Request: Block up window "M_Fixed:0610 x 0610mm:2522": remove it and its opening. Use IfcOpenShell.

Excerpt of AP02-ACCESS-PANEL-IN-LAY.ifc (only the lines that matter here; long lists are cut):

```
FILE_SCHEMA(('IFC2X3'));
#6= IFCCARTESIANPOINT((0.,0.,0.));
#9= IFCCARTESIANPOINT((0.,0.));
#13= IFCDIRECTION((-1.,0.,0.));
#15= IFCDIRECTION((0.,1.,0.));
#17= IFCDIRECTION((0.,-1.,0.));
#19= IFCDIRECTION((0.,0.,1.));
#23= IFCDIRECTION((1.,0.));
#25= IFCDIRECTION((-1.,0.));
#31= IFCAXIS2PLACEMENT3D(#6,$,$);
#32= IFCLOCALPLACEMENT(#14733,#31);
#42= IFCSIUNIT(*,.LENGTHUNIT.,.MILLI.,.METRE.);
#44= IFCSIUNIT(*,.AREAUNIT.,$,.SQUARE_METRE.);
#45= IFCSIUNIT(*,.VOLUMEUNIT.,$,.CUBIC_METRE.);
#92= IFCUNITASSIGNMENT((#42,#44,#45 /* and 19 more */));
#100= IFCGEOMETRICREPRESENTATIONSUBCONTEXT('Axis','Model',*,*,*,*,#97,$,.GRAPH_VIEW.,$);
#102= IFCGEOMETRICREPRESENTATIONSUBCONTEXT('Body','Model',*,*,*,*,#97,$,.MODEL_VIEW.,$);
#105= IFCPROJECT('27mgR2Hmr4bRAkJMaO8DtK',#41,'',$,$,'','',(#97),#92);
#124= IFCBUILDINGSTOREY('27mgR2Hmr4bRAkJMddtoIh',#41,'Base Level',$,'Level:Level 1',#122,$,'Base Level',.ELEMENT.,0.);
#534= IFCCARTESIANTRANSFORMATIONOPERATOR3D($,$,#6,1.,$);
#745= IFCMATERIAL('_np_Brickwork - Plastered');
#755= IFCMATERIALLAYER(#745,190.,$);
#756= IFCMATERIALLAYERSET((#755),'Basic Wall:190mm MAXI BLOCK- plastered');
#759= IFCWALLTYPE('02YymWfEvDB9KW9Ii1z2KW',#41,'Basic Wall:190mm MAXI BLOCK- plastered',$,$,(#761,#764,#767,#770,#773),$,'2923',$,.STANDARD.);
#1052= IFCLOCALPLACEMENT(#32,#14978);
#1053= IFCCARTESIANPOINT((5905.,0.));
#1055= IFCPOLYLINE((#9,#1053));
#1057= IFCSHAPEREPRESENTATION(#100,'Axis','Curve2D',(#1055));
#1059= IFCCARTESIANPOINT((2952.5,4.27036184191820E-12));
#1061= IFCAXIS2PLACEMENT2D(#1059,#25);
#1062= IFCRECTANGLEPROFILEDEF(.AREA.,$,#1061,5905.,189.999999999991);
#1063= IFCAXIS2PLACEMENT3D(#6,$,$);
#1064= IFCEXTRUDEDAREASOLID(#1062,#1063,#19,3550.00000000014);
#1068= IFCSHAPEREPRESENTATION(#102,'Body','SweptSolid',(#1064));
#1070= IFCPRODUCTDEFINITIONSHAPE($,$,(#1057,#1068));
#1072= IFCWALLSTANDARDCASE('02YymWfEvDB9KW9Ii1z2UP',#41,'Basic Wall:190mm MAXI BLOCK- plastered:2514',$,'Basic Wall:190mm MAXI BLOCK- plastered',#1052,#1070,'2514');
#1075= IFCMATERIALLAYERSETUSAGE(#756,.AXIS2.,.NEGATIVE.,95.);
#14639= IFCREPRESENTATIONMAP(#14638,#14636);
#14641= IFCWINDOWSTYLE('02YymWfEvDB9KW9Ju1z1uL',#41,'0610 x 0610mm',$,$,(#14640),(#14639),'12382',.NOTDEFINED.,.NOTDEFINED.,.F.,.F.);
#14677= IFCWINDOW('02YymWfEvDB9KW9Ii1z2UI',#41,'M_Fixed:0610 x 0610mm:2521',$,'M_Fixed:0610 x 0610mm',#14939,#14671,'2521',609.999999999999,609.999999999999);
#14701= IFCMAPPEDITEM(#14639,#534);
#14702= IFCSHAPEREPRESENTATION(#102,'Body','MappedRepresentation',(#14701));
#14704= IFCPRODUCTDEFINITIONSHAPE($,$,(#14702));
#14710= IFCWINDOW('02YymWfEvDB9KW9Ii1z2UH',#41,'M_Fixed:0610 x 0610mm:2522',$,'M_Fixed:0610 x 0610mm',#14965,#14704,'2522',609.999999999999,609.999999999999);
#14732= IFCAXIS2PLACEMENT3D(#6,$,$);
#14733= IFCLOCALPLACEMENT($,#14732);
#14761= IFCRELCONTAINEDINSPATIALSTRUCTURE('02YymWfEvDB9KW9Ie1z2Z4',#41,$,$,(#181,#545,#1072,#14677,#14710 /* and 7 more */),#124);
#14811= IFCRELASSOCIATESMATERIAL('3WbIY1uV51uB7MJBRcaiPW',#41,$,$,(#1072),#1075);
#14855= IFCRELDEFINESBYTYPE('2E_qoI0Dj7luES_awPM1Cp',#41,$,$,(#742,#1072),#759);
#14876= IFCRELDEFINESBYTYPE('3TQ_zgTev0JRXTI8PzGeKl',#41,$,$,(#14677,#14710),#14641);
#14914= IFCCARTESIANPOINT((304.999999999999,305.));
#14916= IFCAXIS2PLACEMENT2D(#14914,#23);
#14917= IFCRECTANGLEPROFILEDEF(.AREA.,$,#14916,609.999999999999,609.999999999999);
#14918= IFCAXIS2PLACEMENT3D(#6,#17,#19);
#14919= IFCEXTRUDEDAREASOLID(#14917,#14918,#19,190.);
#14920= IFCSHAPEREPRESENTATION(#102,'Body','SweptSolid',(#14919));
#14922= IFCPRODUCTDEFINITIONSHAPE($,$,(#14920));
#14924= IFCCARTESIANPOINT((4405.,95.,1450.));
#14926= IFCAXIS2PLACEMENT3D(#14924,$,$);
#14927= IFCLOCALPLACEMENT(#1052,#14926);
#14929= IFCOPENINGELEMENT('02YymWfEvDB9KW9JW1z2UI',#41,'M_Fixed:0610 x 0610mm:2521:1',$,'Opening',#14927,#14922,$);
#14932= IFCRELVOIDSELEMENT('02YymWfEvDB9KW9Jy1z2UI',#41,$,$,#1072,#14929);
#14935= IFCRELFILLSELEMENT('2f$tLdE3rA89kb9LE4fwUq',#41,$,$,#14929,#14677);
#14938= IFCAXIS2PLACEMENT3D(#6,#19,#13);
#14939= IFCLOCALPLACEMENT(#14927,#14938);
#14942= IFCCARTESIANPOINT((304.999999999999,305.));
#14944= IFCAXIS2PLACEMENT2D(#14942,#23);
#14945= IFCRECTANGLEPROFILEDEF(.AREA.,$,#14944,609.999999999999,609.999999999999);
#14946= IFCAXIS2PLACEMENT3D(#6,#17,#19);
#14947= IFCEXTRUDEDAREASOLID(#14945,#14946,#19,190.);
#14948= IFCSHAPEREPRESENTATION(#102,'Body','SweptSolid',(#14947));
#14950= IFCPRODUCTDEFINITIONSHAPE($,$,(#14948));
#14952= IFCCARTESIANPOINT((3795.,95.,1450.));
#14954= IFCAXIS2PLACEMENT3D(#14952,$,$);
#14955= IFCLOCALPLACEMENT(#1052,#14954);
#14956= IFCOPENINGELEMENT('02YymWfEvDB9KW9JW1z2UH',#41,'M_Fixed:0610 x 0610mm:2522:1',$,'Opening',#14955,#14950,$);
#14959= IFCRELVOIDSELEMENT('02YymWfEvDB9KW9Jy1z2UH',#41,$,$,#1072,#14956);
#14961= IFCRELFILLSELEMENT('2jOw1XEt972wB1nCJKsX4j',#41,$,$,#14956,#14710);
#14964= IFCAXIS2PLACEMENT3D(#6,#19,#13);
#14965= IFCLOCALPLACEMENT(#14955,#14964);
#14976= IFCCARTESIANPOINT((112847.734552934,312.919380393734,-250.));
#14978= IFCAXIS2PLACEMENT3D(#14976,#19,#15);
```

```python
import ifcopenshell
import ifcopenshell.api.feature
import ifcopenshell.api.root
import ifcopenshell.geom
import ifcopenshell.util.shape

model = ifcopenshell.open("AP02-ACCESS-PANEL-IN-LAY.ifc")
settings = ifcopenshell.geom.settings()


def volume(element):
    """Net volume in cubic metres, openings subtracted."""
    shape = ifcopenshell.geom.create_shape(settings, element)
    return ifcopenshell.util.shape.get_volume(shape.geometry)


window = model.by_id(14710)
opening = window.FillsVoids[0].RelatingOpeningElement
wall = opening.VoidsElements[0].RelatingBuildingElement
before = volume(wall)

ifcopenshell.api.root.remove_product(model, product=window)
ifcopenshell.api.feature.remove_feature(model, feature=opening)

after = volume(wall)

print(f"wall volume {before:.3f} -> {after:.3f} m3")

model.write("AP02-ACCESS-PANEL-IN-LAY_edited.ifc")
```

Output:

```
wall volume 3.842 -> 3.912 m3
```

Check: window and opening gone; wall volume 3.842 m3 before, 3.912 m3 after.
